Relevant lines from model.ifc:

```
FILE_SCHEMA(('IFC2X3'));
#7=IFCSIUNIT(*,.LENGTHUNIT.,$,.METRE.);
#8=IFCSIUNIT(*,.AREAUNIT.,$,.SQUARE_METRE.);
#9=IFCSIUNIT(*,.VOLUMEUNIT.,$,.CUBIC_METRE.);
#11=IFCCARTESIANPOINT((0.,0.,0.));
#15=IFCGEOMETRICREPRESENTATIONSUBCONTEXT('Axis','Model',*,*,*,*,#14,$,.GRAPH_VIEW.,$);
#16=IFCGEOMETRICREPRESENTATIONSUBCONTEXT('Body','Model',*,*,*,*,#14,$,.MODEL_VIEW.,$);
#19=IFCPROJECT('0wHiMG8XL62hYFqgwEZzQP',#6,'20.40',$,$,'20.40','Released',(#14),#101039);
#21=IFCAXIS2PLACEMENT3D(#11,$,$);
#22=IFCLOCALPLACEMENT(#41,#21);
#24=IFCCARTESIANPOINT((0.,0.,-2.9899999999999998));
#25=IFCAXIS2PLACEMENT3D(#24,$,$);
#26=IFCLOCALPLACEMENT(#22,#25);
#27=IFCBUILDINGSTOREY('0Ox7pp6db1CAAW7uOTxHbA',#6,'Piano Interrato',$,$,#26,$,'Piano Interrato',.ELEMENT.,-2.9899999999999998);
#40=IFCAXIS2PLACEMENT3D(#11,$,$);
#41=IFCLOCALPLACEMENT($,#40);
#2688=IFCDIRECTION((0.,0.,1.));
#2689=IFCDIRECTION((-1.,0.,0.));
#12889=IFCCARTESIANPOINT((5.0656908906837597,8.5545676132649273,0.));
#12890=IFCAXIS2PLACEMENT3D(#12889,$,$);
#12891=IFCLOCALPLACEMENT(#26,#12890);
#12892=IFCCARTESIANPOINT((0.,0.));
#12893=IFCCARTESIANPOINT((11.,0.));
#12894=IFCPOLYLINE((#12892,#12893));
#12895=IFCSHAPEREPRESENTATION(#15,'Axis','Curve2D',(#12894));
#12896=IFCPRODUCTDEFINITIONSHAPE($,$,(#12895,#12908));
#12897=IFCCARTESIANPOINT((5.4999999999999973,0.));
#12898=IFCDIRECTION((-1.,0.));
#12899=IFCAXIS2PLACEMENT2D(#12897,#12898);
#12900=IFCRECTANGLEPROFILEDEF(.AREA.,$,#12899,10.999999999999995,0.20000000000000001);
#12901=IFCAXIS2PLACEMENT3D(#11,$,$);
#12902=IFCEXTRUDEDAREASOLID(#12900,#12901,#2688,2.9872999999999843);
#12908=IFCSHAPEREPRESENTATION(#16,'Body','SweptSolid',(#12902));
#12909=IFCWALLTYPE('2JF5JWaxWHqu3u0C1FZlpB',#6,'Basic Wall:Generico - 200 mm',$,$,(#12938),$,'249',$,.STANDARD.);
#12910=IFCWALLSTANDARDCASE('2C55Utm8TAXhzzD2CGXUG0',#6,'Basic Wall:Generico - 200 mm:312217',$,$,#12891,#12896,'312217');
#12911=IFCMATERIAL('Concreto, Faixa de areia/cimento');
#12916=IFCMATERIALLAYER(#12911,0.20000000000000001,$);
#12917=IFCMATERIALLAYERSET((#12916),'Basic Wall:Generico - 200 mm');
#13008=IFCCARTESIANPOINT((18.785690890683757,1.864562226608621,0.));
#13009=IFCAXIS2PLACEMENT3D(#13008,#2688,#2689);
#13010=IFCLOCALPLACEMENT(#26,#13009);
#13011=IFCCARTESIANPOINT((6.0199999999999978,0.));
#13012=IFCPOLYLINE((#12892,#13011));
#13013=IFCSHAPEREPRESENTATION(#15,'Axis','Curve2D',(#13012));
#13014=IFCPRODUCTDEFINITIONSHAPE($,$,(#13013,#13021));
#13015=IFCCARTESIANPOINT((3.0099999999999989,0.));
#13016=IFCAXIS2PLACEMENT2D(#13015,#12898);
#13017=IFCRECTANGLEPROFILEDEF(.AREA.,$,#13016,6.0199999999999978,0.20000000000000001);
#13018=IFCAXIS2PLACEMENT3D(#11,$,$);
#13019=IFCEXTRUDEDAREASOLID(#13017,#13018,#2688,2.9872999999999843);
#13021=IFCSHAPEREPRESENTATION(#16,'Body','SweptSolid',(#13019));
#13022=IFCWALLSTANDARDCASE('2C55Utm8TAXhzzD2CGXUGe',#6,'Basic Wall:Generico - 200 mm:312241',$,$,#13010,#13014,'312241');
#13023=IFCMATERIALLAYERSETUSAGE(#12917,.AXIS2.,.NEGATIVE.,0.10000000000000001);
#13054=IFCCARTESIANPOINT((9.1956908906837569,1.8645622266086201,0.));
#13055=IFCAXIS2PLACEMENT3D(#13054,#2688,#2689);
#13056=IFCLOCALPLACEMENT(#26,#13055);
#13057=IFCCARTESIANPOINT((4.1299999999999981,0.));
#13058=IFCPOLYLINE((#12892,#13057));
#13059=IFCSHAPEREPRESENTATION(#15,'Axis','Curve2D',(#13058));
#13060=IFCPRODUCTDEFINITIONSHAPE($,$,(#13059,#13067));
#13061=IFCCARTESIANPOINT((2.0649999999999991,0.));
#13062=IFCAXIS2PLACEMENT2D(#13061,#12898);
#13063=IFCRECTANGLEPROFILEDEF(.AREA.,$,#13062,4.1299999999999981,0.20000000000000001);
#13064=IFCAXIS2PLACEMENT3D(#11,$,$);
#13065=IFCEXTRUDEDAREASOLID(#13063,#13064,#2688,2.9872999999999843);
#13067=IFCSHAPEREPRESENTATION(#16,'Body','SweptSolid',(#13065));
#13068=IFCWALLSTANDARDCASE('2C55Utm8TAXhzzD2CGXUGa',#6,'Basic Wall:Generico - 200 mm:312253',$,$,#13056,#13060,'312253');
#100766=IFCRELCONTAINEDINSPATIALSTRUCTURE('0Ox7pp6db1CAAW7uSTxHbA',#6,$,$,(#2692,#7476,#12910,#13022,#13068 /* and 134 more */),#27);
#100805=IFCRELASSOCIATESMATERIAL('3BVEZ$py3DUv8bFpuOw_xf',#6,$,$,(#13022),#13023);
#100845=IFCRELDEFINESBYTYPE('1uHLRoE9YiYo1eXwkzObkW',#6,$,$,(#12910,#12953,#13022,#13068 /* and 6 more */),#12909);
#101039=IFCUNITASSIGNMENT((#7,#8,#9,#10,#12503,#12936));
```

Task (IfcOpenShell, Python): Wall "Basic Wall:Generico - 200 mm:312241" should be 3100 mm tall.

```python
import ifcopenshell
import ifcopenshell.geom
import ifcopenshell.util.representation
import ifcopenshell.util.shape
import ifcopenshell.util.unit

model = ifcopenshell.open("model.ifc")
unit_scale = ifcopenshell.util.unit.calculate_unit_scale(model)
settings = ifcopenshell.geom.settings()


def volume(element):
    """Net volume in cubic metres, openings subtracted."""
    shape = ifcopenshell.geom.create_shape(settings, element)
    return ifcopenshell.util.shape.get_volume(shape.geometry)


wall = model.by_guid("2C55Utm8TAXhzzD2CGXUGe")
before = volume(wall)

body = ifcopenshell.util.representation.get_representation(wall, "Model", "Body")
solid = body.Items[0]
old_height = solid.Depth
solid.Depth = 3.1 / unit_scale
after = volume(wall)

print(f"height {old_height:g} -> {solid.Depth:g}, volume {before:.3f} -> {after:.3f} m3")

model.write("model_updated.ifc")
```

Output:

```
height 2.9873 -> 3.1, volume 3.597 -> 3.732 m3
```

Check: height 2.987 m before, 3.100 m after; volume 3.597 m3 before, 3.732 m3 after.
